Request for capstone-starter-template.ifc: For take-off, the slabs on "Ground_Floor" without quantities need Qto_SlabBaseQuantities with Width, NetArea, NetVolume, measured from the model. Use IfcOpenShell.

First a look at what the model holds.

```python
import ifcopenshell
import ifcopenshell.util.element
import ifcopenshell.util.unit

model = ifcopenshell.open("capstone-starter-template.ifc")
print(model.schema)
for unit_type in ("LENGTHUNIT", "AREAUNIT", "VOLUMEUNIT"):
    print(unit_type, ifcopenshell.util.unit.calculate_unit_scale(model, unit_type))
storey = next(s for s in model.by_type("IfcBuildingStorey") if s.Name == "Ground_Floor")
slabs = [e for e in ifcopenshell.util.element.get_decomposition(storey) if e.is_a("IfcSlab")]
for e in sorted(slabs, key=lambda e: e.id()):
    print(e.id(), e.is_a(), e.Name, list(ifcopenshell.util.element.get_psets(e, qtos_only=True)), sep=" | ")
```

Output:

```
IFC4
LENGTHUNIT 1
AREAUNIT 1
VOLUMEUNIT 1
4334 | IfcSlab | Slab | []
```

```python
import ifcopenshell
import ifcopenshell.api.pset
import ifcopenshell.geom
import ifcopenshell.util.element
import ifcopenshell.util.shape
import ifcopenshell.util.unit

model = ifcopenshell.open("capstone-starter-template.ifc")
unit_scale = ifcopenshell.util.unit.calculate_unit_scale(model)
area_scale = ifcopenshell.util.unit.calculate_unit_scale(model, "AREAUNIT")
volume_scale = ifcopenshell.util.unit.calculate_unit_scale(model, "VOLUMEUNIT")
settings = ifcopenshell.geom.settings()

storey = next(s for s in model.by_type("IfcBuildingStorey") if s.Name == "Ground_Floor")
slabs = [e for e in ifcopenshell.util.element.get_decomposition(storey) if e.is_a("IfcSlab")]

for e in sorted(slabs, key=lambda e: e.id()):
    if ifcopenshell.util.element.get_psets(e, qtos_only=True, should_inherit=False):
        continue
    # Geometry comes back in metres, in the element's own axes.
    shape = ifcopenshell.geom.create_shape(settings, e)
    values = {
        "Width": ifcopenshell.util.shape.get_z(shape.geometry) / unit_scale,
        "NetArea": ifcopenshell.util.shape.get_footprint_area(shape.geometry) / area_scale,
        "NetVolume": ifcopenshell.util.shape.get_volume(shape.geometry) / volume_scale,
    }
    qto = ifcopenshell.api.pset.add_qto(model, product=e, name="Qto_SlabBaseQuantities")
    ifcopenshell.api.pset.edit_qto(model, qto=qto, properties=values)
    print(e.id(), {k: round(v, 3) for k, v in values.items()})

model.write("capstone-starter-template_updated.ifc")
```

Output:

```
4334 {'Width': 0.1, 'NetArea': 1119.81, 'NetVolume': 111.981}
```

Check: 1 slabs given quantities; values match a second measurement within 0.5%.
